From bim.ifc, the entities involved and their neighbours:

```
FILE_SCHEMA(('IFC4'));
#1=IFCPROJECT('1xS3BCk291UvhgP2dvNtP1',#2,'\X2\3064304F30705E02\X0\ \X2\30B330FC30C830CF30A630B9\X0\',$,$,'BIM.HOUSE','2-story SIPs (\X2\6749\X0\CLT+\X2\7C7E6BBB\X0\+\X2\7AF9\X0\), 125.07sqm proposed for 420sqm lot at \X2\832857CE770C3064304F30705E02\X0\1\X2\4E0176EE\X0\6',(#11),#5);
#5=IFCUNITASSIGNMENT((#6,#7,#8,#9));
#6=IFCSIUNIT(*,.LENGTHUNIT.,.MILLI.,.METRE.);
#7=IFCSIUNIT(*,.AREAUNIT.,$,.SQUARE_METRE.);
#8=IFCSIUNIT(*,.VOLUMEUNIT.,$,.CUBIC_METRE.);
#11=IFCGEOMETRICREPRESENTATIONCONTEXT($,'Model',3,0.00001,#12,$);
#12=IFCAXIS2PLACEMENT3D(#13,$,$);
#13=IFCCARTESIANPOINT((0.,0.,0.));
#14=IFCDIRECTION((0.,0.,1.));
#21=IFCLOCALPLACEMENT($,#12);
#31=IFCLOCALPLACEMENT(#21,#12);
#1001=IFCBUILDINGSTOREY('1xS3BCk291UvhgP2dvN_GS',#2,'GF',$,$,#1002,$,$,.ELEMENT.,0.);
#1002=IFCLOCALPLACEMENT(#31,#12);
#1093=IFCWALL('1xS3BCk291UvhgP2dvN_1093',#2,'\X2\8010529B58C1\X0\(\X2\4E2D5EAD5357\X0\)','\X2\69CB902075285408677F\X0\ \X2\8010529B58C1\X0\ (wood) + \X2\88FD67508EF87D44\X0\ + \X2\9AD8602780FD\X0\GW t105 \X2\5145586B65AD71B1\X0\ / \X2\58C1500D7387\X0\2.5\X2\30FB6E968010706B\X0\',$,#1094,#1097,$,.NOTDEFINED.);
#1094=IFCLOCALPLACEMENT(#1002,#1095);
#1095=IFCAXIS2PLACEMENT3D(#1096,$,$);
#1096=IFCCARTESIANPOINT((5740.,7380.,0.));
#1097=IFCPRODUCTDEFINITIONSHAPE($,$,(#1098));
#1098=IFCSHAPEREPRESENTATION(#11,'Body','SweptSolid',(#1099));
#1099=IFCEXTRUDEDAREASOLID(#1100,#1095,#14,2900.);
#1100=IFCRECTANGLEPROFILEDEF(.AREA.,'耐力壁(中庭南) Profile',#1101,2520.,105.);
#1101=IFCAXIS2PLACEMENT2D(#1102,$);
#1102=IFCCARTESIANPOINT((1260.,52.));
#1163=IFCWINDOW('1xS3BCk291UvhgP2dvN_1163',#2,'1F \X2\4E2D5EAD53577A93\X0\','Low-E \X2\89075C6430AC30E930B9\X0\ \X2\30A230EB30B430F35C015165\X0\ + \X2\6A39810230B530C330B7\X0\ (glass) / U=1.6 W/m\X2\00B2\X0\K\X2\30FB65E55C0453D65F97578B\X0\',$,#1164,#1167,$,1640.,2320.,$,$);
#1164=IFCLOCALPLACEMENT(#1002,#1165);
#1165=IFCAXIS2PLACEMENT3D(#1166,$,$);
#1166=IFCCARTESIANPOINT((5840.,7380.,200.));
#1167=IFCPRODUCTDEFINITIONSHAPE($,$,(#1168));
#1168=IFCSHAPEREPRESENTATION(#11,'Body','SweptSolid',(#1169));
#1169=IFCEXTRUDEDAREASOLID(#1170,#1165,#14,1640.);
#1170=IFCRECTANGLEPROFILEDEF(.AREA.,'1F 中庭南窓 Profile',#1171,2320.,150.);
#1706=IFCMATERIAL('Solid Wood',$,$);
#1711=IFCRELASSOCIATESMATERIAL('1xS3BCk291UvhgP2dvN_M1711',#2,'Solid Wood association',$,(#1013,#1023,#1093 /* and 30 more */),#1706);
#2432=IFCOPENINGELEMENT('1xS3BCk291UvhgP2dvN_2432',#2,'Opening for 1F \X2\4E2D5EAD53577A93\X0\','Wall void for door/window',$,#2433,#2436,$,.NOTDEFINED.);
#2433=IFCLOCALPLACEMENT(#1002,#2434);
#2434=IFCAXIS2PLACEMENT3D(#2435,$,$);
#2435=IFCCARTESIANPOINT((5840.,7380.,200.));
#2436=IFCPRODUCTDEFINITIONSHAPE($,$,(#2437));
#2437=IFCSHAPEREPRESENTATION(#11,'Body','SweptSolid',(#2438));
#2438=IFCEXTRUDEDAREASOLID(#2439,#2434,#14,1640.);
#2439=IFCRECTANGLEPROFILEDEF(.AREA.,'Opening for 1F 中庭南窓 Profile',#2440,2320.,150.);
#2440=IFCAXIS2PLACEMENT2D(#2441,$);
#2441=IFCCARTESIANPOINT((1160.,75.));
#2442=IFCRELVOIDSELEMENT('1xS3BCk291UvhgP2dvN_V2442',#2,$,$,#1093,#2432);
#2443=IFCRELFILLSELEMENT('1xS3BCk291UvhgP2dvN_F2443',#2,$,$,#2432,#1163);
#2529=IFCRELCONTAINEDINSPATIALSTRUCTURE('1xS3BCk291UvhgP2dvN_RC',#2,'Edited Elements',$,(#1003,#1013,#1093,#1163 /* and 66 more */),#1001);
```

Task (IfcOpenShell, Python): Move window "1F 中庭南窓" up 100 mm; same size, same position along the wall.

```python
import numpy as np
import ifcopenshell
import ifcopenshell.api.geometry
import ifcopenshell.util.placement
import ifcopenshell.util.unit

model = ifcopenshell.open("bim.ifc")
unit_scale = ifcopenshell.util.unit.calculate_unit_scale(model)

window = model.by_guid("1xS3BCk291UvhgP2dvN_1163")
opening = window.FillsVoids[0].RelatingOpeningElement
dz = 0.1 / unit_scale

shift = np.array([0.0, 0.0, dz])
# The window is not placed relative to its opening, so move both.
for product in (opening, window):
    matrix = ifcopenshell.util.placement.get_local_placement(product.ObjectPlacement)
    matrix[:3, 3] += shift
    ifcopenshell.api.geometry.edit_object_placement(model, product=product, matrix=matrix, is_si=False)

print(f"moved by {dz * unit_scale:+.3f} m")

model.write("bim_edited.ifc")
```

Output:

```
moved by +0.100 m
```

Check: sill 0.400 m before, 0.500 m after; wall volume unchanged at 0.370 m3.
